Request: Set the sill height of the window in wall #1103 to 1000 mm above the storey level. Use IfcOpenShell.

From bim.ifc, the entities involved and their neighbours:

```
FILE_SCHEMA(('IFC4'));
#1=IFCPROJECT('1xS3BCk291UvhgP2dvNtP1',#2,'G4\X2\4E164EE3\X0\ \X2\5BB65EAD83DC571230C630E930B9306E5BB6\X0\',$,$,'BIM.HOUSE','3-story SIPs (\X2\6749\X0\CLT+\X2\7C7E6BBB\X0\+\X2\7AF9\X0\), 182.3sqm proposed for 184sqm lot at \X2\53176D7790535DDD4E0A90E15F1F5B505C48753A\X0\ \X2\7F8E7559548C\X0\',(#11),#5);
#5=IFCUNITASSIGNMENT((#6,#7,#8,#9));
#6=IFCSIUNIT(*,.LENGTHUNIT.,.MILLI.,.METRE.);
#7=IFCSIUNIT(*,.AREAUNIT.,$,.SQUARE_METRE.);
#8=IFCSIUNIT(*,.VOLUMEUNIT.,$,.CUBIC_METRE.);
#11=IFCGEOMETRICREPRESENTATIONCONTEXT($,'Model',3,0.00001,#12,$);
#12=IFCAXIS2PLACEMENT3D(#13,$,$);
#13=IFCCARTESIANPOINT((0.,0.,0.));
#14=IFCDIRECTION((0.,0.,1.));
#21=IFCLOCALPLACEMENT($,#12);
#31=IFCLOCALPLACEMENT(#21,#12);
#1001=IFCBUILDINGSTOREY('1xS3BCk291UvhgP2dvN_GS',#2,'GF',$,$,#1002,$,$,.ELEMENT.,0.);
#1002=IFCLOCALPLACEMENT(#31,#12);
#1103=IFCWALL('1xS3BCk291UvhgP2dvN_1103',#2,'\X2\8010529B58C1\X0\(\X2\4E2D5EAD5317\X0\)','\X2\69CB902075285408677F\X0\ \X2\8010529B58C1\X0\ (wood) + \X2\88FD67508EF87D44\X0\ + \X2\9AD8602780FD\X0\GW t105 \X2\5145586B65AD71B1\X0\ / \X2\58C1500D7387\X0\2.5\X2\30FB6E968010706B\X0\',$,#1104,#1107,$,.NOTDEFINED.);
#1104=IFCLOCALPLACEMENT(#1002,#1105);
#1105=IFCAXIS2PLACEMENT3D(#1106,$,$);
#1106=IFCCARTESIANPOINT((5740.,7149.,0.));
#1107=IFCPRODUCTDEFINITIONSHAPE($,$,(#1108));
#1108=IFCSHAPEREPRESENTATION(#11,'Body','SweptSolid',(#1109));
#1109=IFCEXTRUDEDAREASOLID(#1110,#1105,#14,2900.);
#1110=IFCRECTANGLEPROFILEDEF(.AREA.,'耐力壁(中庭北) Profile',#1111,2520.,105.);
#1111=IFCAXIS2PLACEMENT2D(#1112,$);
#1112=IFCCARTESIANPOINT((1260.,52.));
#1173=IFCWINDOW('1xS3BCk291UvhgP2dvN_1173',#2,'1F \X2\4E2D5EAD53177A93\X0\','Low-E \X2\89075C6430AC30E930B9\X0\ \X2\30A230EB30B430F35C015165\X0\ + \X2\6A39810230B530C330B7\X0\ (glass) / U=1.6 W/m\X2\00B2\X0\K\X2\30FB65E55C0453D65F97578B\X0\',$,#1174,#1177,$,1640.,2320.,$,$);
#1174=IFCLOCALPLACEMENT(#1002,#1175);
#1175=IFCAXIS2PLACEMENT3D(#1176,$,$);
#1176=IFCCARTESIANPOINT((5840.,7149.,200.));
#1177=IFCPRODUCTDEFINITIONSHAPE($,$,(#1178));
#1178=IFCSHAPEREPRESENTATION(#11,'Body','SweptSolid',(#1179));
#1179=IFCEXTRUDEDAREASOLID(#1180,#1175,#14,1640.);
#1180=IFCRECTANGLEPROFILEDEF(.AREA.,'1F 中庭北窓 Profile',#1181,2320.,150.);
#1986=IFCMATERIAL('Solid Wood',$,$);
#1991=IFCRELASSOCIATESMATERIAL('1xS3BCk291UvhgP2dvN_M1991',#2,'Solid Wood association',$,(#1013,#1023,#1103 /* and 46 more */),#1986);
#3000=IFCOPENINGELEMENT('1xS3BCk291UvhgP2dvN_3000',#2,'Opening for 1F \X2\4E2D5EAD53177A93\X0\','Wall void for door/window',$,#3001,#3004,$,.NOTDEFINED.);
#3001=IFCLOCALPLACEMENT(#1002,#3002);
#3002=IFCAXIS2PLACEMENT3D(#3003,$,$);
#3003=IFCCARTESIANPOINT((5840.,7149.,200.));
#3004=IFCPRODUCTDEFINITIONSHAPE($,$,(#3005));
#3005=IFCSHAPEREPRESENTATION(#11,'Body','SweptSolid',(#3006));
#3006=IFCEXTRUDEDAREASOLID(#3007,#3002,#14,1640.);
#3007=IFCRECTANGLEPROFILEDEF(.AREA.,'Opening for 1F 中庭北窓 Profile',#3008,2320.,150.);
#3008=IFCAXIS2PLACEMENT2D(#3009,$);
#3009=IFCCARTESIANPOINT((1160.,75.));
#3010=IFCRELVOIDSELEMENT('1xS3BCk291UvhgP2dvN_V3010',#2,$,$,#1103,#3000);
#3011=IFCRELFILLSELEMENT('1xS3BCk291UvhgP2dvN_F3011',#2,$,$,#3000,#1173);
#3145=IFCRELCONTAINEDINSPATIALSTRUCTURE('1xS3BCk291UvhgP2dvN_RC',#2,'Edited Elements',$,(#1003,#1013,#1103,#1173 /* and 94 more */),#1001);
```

```python
import numpy as np
import ifcopenshell
import ifcopenshell.api.geometry
import ifcopenshell.geom
import ifcopenshell.util.element
import ifcopenshell.util.placement
import ifcopenshell.util.shape
import ifcopenshell.util.unit

model = ifcopenshell.open("bim.ifc")
unit_scale = ifcopenshell.util.unit.calculate_unit_scale(model)

window = model.by_guid("1xS3BCk291UvhgP2dvN_1173")
opening = window.FillsVoids[0].RelatingOpeningElement
storey = ifcopenshell.util.element.get_container(window, ifc_class="IfcBuildingStorey")
level = ifcopenshell.util.placement.get_local_placement(storey.ObjectPlacement)[2, 3]

# The opening's origin need not be at the sill, so measure its lowest point.
shape = ifcopenshell.geom.create_shape(ifcopenshell.geom.settings(), opening)
bottom = ifcopenshell.util.shape.get_shape_bottom_elevation(shape, shape.geometry) / unit_scale
dz = level + 1 / unit_scale - bottom

shift = np.array([0.0, 0.0, dz])
# The window is not placed relative to its opening, so move both.
for product in (opening, window):
    matrix = ifcopenshell.util.placement.get_local_placement(product.ObjectPlacement)
    matrix[:3, 3] += shift
    ifcopenshell.api.geometry.edit_object_placement(model, product=product, matrix=matrix, is_si=False)

print(f"moved by {dz * unit_scale:+.3f} m")

model.write("bim_v2.ifc")
```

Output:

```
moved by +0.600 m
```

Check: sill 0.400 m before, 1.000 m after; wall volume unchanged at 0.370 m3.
